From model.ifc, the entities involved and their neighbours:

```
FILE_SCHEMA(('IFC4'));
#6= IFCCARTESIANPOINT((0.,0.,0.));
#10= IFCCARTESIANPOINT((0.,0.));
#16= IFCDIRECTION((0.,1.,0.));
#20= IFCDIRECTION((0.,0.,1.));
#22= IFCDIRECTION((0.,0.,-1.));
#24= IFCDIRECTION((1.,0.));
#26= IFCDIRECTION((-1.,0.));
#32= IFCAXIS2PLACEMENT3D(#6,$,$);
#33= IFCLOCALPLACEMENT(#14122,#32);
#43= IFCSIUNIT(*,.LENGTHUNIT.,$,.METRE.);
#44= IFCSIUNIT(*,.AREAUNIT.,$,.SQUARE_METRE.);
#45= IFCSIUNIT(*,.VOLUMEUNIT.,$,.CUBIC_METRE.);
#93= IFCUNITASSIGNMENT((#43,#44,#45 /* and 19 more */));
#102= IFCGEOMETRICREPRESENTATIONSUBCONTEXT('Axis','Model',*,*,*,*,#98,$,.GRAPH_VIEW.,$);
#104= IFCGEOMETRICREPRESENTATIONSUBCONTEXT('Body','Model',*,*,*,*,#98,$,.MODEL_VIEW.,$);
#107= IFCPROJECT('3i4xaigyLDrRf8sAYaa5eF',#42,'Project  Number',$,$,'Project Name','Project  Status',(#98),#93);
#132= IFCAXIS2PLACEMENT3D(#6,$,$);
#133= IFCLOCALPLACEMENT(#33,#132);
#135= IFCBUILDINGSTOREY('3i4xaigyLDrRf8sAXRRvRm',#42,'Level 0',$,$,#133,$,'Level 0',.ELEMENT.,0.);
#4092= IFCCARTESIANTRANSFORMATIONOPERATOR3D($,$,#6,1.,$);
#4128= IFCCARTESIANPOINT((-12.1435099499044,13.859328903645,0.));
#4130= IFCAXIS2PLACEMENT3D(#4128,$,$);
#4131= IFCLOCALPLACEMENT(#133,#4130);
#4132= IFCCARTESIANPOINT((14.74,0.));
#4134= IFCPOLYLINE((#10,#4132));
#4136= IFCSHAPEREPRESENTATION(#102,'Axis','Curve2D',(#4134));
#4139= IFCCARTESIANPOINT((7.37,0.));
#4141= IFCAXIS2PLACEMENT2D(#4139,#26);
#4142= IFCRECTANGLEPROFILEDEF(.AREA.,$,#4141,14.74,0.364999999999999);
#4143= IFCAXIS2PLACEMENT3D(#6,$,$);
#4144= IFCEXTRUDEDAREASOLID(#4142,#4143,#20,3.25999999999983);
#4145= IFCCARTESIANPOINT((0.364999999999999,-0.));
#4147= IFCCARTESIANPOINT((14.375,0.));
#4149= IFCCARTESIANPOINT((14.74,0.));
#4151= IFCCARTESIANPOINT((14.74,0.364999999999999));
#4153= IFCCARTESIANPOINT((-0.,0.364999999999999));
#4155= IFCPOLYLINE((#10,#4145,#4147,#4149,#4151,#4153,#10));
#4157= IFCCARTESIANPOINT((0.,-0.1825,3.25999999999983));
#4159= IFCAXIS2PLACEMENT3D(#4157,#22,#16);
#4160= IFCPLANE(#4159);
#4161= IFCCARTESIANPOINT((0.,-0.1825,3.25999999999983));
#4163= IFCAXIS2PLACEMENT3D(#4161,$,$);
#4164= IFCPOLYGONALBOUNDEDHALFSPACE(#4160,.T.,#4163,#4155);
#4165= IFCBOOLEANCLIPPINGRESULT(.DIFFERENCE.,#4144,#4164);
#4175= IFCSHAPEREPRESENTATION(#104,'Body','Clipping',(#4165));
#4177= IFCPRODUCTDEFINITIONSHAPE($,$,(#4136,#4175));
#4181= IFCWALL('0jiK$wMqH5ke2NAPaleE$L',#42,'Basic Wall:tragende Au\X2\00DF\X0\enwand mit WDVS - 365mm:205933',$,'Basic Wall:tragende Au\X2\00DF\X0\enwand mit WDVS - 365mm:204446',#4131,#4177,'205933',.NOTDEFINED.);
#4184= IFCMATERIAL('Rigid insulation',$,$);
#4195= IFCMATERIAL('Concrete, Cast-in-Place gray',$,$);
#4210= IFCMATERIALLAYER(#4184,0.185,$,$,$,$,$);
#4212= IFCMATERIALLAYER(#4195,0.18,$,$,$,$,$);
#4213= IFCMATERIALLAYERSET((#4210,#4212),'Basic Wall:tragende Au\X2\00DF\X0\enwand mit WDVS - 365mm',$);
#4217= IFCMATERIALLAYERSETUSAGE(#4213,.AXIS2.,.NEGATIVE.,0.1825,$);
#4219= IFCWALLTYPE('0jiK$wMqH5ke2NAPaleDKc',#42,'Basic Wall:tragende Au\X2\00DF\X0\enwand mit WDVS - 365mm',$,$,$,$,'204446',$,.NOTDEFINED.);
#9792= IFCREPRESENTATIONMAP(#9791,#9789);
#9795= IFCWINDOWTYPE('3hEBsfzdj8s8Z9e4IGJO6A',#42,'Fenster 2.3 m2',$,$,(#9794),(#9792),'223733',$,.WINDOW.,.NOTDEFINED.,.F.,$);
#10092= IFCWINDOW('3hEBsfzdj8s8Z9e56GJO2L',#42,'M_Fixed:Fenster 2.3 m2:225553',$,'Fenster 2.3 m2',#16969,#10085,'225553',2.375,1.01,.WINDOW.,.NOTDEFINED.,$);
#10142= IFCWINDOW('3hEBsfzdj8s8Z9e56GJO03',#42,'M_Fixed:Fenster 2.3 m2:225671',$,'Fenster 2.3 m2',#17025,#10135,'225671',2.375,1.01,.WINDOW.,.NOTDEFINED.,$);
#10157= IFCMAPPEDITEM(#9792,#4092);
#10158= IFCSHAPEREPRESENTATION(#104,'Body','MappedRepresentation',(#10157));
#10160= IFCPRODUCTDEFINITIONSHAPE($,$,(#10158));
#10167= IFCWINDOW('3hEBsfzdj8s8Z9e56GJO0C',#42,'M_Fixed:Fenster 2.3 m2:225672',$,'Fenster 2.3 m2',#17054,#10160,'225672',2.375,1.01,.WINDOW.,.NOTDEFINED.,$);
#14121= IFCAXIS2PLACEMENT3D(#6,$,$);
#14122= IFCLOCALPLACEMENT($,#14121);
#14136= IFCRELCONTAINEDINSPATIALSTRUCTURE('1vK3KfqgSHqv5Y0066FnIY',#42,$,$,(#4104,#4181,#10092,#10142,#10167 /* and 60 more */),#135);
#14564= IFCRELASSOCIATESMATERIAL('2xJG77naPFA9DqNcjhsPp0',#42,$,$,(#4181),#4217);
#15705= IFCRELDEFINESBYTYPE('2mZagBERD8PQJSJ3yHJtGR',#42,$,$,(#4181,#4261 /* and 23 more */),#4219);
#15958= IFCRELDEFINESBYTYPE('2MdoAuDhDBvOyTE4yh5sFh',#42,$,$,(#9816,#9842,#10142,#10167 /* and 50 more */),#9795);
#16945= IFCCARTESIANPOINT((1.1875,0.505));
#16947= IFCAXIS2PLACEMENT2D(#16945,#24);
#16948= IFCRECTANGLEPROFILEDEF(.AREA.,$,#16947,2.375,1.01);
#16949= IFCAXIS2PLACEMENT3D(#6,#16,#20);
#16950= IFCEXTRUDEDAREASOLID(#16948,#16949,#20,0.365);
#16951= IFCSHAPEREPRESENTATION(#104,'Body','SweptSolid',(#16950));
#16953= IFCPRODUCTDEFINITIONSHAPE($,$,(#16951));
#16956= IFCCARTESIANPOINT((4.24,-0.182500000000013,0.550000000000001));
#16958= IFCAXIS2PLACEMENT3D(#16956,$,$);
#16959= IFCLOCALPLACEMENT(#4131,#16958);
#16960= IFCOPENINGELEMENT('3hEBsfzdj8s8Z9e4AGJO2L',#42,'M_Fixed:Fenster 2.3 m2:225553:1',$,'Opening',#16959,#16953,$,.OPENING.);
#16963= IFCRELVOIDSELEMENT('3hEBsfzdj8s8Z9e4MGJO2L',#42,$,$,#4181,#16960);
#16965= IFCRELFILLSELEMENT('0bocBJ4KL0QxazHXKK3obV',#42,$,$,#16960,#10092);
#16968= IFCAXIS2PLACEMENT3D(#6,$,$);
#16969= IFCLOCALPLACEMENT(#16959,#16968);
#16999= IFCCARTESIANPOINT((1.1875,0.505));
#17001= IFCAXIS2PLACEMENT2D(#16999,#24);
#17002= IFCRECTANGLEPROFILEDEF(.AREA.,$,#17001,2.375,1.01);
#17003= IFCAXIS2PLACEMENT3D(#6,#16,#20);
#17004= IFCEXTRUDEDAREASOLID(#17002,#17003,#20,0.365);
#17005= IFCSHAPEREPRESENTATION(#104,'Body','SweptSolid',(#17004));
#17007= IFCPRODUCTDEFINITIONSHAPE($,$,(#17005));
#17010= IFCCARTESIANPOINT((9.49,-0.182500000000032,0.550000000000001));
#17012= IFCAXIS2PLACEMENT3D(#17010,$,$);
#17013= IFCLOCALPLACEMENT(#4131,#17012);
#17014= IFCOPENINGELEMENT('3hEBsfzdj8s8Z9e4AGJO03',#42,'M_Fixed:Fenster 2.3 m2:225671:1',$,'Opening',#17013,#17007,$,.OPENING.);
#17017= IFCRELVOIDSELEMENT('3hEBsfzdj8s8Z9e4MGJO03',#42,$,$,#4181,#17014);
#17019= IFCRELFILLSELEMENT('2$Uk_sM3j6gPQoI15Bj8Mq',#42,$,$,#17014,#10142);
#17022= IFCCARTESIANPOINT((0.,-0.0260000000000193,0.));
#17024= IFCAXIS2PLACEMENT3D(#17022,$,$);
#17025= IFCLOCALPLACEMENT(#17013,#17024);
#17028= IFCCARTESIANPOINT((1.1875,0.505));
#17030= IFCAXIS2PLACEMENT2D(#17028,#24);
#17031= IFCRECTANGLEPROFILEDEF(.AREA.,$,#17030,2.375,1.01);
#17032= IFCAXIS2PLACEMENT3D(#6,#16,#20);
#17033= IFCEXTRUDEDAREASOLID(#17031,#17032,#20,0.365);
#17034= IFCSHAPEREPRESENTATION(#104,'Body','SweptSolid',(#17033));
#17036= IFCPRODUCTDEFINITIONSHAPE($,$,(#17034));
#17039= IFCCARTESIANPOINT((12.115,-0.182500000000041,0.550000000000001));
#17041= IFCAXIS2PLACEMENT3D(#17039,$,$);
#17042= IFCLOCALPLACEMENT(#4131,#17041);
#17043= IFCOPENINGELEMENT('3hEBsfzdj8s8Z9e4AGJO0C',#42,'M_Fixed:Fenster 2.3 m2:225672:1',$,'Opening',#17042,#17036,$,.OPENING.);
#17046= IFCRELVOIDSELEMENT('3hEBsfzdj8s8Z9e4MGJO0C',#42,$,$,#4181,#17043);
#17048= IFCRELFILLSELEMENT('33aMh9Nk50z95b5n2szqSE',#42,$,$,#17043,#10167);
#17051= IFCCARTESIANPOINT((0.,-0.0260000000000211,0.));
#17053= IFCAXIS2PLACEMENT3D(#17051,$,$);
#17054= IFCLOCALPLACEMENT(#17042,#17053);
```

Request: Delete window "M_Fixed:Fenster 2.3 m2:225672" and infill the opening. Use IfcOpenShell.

```python
import ifcopenshell
import ifcopenshell.api.feature
import ifcopenshell.api.root
import ifcopenshell.geom
import ifcopenshell.util.shape

model = ifcopenshell.open("model.ifc")
settings = ifcopenshell.geom.settings()


def volume(element):
    """Net volume in cubic metres, openings subtracted."""
    shape = ifcopenshell.geom.create_shape(settings, element)
    return ifcopenshell.util.shape.get_volume(shape.geometry)


window = model.by_guid("3hEBsfzdj8s8Z9e56GJO0C")
opening = window.FillsVoids[0].RelatingOpeningElement
wall = opening.VoidsElements[0].RelatingBuildingElement
before = volume(wall)

ifcopenshell.api.root.remove_product(model, product=window)
ifcopenshell.api.feature.remove_feature(model, feature=opening)

after = volume(wall)

print(f"wall volume {before:.3f} -> {after:.3f} m3")

model.write("model_edited.ifc")
```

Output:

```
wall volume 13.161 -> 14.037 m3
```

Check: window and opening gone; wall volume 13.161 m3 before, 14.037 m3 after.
